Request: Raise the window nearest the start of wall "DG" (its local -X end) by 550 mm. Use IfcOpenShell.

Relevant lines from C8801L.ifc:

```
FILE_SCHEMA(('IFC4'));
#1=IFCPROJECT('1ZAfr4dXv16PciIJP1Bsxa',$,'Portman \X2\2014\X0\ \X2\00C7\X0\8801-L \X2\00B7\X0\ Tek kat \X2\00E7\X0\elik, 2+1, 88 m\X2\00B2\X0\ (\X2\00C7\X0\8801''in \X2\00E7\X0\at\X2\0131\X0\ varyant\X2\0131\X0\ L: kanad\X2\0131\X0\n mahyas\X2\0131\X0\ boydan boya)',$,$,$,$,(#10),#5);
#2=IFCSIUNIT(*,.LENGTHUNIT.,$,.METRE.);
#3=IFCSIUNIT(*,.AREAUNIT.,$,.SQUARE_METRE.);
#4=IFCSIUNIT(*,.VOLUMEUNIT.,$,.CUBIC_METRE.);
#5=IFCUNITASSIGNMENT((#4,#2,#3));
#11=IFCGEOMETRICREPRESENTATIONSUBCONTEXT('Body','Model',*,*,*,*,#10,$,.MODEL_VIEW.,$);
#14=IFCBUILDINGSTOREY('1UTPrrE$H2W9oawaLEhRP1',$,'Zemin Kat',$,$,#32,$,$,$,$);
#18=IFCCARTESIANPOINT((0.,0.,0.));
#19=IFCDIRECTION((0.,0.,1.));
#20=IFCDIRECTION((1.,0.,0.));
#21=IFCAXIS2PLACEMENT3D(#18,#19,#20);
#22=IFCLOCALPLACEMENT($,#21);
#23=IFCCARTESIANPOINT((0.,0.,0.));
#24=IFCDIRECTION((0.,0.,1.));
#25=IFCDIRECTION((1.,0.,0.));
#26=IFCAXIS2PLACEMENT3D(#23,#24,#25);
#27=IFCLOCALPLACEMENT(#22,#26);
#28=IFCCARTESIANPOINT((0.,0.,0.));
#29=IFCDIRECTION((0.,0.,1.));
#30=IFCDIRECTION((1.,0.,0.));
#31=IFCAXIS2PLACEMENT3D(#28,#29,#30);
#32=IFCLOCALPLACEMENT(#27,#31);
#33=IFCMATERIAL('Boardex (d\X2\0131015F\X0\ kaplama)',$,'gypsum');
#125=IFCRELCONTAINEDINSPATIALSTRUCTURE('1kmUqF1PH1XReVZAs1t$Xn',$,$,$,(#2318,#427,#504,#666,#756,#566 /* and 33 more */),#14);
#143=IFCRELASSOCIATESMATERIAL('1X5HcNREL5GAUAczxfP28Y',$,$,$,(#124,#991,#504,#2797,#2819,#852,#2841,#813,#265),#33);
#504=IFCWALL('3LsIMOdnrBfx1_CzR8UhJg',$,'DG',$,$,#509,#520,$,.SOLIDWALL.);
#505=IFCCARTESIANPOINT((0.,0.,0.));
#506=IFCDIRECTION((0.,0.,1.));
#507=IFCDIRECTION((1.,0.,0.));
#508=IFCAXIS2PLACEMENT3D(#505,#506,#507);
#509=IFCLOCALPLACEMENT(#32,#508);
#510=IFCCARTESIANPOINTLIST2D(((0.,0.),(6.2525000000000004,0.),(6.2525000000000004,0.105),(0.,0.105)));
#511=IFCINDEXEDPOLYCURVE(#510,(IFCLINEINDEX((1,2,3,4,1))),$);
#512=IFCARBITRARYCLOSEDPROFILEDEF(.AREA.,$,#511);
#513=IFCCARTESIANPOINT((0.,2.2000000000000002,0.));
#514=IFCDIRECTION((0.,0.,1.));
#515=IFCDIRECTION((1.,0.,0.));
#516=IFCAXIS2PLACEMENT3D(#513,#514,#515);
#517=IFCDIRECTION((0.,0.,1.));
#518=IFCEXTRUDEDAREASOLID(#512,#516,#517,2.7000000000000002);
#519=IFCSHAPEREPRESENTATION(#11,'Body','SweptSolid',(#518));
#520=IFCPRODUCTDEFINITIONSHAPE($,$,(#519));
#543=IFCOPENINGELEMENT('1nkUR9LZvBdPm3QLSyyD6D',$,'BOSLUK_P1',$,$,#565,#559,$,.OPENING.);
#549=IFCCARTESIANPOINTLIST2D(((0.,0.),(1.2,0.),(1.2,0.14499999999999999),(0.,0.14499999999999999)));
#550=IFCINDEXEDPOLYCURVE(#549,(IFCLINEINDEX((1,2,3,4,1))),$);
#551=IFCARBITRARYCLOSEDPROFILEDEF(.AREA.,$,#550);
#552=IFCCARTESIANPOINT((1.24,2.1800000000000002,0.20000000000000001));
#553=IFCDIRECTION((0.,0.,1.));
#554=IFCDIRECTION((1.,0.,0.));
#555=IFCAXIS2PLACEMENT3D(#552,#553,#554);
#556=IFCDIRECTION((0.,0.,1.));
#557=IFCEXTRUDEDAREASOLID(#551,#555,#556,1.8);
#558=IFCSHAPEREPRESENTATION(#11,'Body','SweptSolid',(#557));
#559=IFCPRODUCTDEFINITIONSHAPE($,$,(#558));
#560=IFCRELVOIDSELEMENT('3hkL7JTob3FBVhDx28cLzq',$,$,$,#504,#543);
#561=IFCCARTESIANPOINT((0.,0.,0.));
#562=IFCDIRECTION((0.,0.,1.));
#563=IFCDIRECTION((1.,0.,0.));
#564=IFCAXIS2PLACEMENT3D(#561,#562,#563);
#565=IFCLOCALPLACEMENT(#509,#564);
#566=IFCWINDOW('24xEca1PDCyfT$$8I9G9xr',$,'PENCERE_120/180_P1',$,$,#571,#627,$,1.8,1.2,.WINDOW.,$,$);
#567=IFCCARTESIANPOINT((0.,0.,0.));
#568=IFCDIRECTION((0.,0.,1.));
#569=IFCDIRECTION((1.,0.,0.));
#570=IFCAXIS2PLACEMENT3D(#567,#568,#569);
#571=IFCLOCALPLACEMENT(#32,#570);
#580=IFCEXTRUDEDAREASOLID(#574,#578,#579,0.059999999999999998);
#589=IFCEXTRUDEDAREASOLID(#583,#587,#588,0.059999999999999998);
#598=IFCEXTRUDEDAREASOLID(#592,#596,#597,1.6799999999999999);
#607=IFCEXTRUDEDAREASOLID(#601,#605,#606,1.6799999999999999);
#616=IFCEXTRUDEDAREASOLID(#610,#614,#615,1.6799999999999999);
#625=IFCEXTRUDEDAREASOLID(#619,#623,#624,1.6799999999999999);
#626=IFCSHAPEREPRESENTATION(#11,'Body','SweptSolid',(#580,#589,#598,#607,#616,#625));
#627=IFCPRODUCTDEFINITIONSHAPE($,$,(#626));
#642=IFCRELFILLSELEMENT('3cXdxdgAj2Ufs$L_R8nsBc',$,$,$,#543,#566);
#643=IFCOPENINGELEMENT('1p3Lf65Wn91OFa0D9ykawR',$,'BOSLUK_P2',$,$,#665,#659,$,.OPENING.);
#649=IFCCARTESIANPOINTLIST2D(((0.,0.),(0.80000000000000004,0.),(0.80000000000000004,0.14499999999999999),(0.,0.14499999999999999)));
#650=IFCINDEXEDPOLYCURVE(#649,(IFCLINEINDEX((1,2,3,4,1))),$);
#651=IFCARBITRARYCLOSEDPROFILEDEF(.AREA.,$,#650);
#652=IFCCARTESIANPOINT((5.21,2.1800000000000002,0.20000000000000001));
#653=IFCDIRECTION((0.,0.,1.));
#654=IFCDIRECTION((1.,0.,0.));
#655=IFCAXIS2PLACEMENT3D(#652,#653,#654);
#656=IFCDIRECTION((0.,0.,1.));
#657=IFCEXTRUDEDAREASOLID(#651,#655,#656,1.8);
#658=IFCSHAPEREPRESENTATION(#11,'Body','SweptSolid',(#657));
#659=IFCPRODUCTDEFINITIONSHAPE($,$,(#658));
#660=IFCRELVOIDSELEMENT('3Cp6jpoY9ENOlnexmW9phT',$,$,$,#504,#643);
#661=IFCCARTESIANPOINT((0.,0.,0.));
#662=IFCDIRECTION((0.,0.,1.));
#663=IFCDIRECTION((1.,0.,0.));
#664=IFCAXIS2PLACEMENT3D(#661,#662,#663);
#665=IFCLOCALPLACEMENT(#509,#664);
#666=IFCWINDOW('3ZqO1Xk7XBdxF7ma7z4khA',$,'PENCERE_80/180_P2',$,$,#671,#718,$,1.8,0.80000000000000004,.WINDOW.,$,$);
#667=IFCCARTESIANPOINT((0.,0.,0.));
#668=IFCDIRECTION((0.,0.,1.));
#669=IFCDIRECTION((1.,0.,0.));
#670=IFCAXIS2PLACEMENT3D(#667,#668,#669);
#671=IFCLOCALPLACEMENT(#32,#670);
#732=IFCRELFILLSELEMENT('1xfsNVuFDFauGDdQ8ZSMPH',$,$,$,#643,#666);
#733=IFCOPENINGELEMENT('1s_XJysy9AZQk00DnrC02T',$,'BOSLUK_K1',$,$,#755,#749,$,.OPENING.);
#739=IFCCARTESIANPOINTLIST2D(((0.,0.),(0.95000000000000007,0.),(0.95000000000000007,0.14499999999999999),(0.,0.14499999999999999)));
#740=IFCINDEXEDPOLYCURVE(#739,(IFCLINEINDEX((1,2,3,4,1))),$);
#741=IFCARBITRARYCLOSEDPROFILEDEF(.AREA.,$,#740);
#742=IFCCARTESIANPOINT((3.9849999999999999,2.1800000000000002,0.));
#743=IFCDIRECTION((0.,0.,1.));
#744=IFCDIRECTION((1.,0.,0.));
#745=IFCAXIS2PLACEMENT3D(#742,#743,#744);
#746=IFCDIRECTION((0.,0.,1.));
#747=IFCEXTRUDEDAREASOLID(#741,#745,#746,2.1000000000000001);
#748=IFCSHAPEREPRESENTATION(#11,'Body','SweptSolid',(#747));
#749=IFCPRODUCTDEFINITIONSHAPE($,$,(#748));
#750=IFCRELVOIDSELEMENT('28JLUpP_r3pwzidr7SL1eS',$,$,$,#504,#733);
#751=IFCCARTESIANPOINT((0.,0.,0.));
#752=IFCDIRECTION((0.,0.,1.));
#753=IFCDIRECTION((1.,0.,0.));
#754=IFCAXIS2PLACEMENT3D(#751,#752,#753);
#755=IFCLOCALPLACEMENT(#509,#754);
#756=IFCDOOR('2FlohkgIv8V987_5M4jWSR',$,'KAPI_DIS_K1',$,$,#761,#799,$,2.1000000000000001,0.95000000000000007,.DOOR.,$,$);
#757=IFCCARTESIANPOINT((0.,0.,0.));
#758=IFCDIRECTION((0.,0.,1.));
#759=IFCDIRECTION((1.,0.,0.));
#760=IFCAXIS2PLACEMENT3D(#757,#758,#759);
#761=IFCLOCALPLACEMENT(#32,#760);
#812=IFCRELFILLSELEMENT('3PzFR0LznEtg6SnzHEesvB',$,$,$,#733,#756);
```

```python
import numpy as np
import ifcopenshell
import ifcopenshell.api.geometry
import ifcopenshell.util.placement
import ifcopenshell.util.unit

model = ifcopenshell.open("C8801L.ifc")
unit_scale = ifcopenshell.util.unit.calculate_unit_scale(model)

window = model.by_guid("24xEca1PDCyfT$$8I9G9xr")
opening = window.FillsVoids[0].RelatingOpeningElement
dz = 0.55

shift = np.array([0.0, 0.0, dz])
# The window is not placed relative to its opening, so move both.
for product in (opening, window):
    matrix = ifcopenshell.util.placement.get_local_placement(product.ObjectPlacement)
    matrix[:3, 3] += shift
    ifcopenshell.api.geometry.edit_object_placement(model, product=product, matrix=matrix, is_si=False)

print(f"moved by {dz * unit_scale:+.3f} m")

model.write("C8801L_updated.ifc")
```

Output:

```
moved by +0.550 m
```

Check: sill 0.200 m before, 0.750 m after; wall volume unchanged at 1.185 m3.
